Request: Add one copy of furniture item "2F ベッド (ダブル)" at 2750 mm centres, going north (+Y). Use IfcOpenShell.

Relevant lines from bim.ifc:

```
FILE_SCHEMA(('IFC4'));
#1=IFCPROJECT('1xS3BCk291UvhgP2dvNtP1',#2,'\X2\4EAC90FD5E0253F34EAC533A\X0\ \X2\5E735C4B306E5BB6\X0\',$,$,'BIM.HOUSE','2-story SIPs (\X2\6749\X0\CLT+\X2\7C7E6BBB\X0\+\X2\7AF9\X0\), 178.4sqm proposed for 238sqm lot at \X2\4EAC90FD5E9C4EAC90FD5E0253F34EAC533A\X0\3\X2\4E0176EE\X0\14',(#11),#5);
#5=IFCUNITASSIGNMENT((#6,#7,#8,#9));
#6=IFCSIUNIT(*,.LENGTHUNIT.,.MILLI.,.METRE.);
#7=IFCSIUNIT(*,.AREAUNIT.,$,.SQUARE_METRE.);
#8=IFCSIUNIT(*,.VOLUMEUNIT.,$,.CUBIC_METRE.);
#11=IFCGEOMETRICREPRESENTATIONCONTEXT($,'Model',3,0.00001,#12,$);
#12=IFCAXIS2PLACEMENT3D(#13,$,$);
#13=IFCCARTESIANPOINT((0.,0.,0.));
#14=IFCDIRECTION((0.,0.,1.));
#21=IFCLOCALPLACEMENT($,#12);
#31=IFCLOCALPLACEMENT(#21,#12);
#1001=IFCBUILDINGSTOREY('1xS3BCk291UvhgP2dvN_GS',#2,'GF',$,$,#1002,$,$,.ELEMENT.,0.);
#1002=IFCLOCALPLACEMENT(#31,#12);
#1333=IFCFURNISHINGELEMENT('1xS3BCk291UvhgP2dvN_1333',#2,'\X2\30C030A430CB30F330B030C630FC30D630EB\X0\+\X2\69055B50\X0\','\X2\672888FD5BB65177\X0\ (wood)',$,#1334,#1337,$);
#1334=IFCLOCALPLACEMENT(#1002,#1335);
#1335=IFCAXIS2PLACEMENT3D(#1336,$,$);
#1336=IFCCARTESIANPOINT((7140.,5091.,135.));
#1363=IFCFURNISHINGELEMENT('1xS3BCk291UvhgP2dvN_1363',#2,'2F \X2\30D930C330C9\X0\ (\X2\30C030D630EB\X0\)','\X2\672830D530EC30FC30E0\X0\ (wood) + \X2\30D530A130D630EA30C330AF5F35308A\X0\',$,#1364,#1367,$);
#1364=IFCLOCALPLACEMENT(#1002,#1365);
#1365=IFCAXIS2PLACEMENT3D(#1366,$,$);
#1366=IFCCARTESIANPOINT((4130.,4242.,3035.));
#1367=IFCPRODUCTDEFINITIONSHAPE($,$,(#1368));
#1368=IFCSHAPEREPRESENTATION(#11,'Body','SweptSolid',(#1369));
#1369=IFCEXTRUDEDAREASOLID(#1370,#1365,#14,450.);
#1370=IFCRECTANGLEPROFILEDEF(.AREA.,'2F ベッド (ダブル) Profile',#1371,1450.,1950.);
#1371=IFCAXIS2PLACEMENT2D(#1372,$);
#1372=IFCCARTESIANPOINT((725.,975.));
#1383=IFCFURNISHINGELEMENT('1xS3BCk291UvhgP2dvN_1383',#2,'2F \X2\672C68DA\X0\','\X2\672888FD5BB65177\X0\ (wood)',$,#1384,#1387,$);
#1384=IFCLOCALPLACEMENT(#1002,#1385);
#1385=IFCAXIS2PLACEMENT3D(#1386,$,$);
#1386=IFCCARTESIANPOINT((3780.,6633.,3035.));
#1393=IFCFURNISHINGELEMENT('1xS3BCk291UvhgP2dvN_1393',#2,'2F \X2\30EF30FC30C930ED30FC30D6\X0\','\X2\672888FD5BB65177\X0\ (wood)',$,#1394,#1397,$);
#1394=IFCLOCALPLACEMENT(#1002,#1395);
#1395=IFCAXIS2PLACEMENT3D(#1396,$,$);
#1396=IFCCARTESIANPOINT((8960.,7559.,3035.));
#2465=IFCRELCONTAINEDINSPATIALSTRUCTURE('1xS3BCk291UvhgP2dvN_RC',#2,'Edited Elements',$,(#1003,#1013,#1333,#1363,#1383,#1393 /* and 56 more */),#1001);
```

```python
import numpy as np
import ifcopenshell
import ifcopenshell.api.geometry
import ifcopenshell.api.root
import ifcopenshell.util.element
import ifcopenshell.util.placement

model = ifcopenshell.open("bim.ifc")


def reuse_history(source, copy):
    """copy_class also copies each property set's owner history, people and application; keep the originals."""
    for rel in copy.IsDefinedBy:
        if rel.is_a("IfcRelDefinesByProperties") and (history := rel.RelatingPropertyDefinition.OwnerHistory):
            rel.RelatingPropertyDefinition.OwnerHistory = source.OwnerHistory
            ifcopenshell.util.element.remove_deep2(model, history)


source = model.by_guid("1xS3BCk291UvhgP2dvN_1363")
base = ifcopenshell.util.placement.get_local_placement(source.ObjectPlacement)
step = np.array([0.0, 1.0, 0.0]) * 2750.0

for i in range(1, 2):
    copy = ifcopenshell.api.root.copy_class(model, product=source)
    copy.Representation = ifcopenshell.util.element.copy_deep(
        model, source.Representation, exclude=["IfcGeometricRepresentationContext", "IfcRepresentationMap"]
    )
    reuse_history(source, copy)
    matrix = base.copy()
    matrix[:3, 3] += i * step
    print("added at", matrix[:3, 3].round(3) + 0.0)
    ifcopenshell.api.geometry.edit_object_placement(model, product=copy, matrix=matrix, is_si=False)

model.write("bim_updated.ifc")
```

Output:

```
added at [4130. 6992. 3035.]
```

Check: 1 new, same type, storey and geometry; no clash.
